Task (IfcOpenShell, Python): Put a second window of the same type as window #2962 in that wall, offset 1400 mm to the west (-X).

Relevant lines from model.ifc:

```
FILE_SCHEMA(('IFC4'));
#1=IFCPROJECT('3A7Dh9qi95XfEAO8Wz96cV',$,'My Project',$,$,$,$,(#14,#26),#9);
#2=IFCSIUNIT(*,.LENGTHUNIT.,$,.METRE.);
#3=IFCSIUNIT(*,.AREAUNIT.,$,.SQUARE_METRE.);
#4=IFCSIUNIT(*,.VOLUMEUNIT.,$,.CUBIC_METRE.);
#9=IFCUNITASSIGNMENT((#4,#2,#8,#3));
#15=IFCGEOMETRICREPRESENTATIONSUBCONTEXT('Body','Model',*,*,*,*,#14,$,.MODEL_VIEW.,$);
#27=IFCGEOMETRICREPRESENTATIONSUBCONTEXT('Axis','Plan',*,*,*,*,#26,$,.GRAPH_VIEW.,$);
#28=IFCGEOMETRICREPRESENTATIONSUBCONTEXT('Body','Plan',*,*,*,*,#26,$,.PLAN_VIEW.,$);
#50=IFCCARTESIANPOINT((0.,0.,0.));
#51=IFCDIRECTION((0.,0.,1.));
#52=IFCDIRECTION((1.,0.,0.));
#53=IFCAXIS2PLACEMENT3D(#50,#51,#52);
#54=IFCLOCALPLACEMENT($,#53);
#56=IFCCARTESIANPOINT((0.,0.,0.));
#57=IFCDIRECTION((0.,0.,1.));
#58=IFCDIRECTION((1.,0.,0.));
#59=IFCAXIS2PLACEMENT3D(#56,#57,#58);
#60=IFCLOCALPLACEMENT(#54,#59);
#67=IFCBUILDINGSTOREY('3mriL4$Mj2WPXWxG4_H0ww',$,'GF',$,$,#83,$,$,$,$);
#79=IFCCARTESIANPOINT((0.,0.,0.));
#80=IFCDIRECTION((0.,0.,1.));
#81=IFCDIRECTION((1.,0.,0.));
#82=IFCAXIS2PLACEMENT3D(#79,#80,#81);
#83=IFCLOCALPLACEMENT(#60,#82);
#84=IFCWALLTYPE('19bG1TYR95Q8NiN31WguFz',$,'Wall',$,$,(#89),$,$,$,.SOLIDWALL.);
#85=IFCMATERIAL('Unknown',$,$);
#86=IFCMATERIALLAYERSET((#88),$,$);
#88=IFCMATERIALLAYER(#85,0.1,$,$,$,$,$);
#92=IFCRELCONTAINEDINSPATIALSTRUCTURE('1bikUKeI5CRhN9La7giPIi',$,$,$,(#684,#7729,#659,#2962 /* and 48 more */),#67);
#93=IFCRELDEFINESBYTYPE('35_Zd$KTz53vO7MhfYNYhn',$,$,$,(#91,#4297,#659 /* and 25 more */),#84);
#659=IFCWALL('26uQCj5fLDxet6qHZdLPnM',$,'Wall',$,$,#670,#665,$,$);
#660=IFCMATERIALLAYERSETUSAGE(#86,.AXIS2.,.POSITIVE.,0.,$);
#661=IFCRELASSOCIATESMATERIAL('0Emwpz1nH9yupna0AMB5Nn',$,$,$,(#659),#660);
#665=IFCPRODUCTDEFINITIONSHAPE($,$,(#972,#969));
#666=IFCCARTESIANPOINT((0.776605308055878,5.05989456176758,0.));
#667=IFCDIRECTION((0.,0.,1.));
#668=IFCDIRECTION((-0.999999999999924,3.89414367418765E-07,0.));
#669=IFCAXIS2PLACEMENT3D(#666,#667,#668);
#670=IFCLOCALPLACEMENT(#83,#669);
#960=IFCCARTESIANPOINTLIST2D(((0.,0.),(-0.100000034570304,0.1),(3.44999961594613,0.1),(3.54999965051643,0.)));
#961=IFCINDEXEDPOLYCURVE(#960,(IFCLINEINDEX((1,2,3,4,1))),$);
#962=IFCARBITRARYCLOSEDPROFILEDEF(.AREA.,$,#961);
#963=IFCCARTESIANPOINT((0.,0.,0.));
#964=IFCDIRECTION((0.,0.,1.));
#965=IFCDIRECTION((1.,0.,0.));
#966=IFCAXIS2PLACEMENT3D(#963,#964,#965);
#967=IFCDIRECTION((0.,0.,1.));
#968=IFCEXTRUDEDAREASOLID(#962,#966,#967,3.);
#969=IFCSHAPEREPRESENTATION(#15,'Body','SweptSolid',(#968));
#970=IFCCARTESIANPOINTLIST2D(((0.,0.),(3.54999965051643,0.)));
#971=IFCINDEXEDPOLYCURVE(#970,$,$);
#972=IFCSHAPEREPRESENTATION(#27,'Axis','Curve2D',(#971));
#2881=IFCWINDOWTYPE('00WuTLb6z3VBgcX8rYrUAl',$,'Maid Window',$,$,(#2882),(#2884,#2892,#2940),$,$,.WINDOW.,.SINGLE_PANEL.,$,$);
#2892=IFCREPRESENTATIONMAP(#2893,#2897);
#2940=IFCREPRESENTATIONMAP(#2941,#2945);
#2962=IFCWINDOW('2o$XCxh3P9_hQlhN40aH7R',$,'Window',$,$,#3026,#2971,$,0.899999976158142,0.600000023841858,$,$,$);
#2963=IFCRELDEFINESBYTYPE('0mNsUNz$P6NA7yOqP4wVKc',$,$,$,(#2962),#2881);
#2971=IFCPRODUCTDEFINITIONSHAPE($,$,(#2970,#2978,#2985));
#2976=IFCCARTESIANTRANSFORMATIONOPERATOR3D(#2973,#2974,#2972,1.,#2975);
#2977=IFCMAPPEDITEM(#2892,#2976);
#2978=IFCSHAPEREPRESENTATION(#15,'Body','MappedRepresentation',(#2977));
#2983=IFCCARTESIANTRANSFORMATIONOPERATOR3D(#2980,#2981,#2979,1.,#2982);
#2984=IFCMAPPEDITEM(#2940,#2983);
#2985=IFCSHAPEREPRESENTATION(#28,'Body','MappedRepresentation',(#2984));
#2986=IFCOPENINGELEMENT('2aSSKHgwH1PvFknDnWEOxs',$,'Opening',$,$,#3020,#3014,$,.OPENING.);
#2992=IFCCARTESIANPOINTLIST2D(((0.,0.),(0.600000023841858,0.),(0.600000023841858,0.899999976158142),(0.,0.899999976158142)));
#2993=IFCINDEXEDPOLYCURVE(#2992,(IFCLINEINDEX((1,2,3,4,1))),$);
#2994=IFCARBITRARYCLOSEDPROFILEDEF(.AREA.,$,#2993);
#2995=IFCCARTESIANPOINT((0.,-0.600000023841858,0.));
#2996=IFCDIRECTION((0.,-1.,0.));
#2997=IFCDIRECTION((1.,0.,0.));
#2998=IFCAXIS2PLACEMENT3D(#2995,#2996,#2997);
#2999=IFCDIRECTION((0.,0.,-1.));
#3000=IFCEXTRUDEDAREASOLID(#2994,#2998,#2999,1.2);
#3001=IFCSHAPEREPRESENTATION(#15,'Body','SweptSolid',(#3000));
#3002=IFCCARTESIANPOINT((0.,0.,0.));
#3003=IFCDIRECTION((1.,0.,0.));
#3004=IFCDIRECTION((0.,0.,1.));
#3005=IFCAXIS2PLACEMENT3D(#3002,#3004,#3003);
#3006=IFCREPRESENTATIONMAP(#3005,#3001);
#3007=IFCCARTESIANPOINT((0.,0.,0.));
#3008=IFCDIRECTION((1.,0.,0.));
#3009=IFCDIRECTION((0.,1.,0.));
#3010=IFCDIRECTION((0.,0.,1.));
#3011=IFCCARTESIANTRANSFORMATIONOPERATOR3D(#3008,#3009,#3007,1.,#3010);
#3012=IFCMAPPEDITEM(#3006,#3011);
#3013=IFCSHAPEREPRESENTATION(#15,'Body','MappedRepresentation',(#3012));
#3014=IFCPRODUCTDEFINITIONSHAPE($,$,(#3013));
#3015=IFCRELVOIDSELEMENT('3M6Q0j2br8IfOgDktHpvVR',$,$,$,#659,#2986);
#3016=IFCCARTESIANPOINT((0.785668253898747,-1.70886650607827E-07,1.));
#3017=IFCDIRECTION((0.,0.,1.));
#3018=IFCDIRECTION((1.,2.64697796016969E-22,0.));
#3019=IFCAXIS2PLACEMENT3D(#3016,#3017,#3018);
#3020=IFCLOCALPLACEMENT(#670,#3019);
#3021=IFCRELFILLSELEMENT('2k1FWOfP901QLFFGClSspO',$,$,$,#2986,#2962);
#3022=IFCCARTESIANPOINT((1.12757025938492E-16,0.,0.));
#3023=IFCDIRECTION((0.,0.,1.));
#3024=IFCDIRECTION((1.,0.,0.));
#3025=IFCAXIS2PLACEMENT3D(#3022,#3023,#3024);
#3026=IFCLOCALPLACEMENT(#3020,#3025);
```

```python
import ifcopenshell
import ifcopenshell.api.feature
import ifcopenshell.api.geometry
import ifcopenshell.api.root
import ifcopenshell.geom
import ifcopenshell.util.element
import ifcopenshell.util.placement
import ifcopenshell.util.shape
import ifcopenshell.util.unit

model = ifcopenshell.open("model.ifc")
unit_scale = ifcopenshell.util.unit.calculate_unit_scale(model)
settings = ifcopenshell.geom.settings()


def volume(element):
    """Net volume in cubic metres, openings subtracted."""
    shape = ifcopenshell.geom.create_shape(settings, element)
    return ifcopenshell.util.shape.get_volume(shape.geometry)


window = model.by_id(2962)
opening = window.FillsVoids[0].RelatingOpeningElement
wall = opening.VoidsElements[0].RelatingBuildingElement
before = volume(wall)
shift = ifcopenshell.util.placement.get_local_placement(wall.ObjectPlacement)[:3, 0] * 1.4 / unit_scale

# copy_class copies the void relationship, type, container and properties, but no geometry.
new_opening = ifcopenshell.api.root.copy_class(model, product=opening)
new_opening.Representation = ifcopenshell.util.element.copy_deep(
    model, opening.Representation, exclude=["IfcGeometricRepresentationContext", "IfcRepresentationMap"]
)
new_window = ifcopenshell.api.root.copy_class(model, product=window)
new_window.Representation = ifcopenshell.util.element.copy_deep(
    model, window.Representation, exclude=["IfcGeometricRepresentationContext", "IfcRepresentationMap"]
)
ifcopenshell.api.feature.add_filling(model, opening=new_opening, element=new_window)

for old, new in ((opening, new_opening), (window, new_window)):
    matrix = ifcopenshell.util.placement.get_local_placement(old.ObjectPlacement)
    matrix[:3, 3] += shift
    ifcopenshell.api.geometry.edit_object_placement(model, product=new, matrix=matrix, is_si=False)

after = volume(wall)

print(f"wall volume {before:.3f} -> {after:.3f} m3")

model.write("model-out.ifc")
```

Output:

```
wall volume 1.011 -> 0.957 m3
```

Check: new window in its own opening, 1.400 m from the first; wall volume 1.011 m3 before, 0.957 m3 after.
